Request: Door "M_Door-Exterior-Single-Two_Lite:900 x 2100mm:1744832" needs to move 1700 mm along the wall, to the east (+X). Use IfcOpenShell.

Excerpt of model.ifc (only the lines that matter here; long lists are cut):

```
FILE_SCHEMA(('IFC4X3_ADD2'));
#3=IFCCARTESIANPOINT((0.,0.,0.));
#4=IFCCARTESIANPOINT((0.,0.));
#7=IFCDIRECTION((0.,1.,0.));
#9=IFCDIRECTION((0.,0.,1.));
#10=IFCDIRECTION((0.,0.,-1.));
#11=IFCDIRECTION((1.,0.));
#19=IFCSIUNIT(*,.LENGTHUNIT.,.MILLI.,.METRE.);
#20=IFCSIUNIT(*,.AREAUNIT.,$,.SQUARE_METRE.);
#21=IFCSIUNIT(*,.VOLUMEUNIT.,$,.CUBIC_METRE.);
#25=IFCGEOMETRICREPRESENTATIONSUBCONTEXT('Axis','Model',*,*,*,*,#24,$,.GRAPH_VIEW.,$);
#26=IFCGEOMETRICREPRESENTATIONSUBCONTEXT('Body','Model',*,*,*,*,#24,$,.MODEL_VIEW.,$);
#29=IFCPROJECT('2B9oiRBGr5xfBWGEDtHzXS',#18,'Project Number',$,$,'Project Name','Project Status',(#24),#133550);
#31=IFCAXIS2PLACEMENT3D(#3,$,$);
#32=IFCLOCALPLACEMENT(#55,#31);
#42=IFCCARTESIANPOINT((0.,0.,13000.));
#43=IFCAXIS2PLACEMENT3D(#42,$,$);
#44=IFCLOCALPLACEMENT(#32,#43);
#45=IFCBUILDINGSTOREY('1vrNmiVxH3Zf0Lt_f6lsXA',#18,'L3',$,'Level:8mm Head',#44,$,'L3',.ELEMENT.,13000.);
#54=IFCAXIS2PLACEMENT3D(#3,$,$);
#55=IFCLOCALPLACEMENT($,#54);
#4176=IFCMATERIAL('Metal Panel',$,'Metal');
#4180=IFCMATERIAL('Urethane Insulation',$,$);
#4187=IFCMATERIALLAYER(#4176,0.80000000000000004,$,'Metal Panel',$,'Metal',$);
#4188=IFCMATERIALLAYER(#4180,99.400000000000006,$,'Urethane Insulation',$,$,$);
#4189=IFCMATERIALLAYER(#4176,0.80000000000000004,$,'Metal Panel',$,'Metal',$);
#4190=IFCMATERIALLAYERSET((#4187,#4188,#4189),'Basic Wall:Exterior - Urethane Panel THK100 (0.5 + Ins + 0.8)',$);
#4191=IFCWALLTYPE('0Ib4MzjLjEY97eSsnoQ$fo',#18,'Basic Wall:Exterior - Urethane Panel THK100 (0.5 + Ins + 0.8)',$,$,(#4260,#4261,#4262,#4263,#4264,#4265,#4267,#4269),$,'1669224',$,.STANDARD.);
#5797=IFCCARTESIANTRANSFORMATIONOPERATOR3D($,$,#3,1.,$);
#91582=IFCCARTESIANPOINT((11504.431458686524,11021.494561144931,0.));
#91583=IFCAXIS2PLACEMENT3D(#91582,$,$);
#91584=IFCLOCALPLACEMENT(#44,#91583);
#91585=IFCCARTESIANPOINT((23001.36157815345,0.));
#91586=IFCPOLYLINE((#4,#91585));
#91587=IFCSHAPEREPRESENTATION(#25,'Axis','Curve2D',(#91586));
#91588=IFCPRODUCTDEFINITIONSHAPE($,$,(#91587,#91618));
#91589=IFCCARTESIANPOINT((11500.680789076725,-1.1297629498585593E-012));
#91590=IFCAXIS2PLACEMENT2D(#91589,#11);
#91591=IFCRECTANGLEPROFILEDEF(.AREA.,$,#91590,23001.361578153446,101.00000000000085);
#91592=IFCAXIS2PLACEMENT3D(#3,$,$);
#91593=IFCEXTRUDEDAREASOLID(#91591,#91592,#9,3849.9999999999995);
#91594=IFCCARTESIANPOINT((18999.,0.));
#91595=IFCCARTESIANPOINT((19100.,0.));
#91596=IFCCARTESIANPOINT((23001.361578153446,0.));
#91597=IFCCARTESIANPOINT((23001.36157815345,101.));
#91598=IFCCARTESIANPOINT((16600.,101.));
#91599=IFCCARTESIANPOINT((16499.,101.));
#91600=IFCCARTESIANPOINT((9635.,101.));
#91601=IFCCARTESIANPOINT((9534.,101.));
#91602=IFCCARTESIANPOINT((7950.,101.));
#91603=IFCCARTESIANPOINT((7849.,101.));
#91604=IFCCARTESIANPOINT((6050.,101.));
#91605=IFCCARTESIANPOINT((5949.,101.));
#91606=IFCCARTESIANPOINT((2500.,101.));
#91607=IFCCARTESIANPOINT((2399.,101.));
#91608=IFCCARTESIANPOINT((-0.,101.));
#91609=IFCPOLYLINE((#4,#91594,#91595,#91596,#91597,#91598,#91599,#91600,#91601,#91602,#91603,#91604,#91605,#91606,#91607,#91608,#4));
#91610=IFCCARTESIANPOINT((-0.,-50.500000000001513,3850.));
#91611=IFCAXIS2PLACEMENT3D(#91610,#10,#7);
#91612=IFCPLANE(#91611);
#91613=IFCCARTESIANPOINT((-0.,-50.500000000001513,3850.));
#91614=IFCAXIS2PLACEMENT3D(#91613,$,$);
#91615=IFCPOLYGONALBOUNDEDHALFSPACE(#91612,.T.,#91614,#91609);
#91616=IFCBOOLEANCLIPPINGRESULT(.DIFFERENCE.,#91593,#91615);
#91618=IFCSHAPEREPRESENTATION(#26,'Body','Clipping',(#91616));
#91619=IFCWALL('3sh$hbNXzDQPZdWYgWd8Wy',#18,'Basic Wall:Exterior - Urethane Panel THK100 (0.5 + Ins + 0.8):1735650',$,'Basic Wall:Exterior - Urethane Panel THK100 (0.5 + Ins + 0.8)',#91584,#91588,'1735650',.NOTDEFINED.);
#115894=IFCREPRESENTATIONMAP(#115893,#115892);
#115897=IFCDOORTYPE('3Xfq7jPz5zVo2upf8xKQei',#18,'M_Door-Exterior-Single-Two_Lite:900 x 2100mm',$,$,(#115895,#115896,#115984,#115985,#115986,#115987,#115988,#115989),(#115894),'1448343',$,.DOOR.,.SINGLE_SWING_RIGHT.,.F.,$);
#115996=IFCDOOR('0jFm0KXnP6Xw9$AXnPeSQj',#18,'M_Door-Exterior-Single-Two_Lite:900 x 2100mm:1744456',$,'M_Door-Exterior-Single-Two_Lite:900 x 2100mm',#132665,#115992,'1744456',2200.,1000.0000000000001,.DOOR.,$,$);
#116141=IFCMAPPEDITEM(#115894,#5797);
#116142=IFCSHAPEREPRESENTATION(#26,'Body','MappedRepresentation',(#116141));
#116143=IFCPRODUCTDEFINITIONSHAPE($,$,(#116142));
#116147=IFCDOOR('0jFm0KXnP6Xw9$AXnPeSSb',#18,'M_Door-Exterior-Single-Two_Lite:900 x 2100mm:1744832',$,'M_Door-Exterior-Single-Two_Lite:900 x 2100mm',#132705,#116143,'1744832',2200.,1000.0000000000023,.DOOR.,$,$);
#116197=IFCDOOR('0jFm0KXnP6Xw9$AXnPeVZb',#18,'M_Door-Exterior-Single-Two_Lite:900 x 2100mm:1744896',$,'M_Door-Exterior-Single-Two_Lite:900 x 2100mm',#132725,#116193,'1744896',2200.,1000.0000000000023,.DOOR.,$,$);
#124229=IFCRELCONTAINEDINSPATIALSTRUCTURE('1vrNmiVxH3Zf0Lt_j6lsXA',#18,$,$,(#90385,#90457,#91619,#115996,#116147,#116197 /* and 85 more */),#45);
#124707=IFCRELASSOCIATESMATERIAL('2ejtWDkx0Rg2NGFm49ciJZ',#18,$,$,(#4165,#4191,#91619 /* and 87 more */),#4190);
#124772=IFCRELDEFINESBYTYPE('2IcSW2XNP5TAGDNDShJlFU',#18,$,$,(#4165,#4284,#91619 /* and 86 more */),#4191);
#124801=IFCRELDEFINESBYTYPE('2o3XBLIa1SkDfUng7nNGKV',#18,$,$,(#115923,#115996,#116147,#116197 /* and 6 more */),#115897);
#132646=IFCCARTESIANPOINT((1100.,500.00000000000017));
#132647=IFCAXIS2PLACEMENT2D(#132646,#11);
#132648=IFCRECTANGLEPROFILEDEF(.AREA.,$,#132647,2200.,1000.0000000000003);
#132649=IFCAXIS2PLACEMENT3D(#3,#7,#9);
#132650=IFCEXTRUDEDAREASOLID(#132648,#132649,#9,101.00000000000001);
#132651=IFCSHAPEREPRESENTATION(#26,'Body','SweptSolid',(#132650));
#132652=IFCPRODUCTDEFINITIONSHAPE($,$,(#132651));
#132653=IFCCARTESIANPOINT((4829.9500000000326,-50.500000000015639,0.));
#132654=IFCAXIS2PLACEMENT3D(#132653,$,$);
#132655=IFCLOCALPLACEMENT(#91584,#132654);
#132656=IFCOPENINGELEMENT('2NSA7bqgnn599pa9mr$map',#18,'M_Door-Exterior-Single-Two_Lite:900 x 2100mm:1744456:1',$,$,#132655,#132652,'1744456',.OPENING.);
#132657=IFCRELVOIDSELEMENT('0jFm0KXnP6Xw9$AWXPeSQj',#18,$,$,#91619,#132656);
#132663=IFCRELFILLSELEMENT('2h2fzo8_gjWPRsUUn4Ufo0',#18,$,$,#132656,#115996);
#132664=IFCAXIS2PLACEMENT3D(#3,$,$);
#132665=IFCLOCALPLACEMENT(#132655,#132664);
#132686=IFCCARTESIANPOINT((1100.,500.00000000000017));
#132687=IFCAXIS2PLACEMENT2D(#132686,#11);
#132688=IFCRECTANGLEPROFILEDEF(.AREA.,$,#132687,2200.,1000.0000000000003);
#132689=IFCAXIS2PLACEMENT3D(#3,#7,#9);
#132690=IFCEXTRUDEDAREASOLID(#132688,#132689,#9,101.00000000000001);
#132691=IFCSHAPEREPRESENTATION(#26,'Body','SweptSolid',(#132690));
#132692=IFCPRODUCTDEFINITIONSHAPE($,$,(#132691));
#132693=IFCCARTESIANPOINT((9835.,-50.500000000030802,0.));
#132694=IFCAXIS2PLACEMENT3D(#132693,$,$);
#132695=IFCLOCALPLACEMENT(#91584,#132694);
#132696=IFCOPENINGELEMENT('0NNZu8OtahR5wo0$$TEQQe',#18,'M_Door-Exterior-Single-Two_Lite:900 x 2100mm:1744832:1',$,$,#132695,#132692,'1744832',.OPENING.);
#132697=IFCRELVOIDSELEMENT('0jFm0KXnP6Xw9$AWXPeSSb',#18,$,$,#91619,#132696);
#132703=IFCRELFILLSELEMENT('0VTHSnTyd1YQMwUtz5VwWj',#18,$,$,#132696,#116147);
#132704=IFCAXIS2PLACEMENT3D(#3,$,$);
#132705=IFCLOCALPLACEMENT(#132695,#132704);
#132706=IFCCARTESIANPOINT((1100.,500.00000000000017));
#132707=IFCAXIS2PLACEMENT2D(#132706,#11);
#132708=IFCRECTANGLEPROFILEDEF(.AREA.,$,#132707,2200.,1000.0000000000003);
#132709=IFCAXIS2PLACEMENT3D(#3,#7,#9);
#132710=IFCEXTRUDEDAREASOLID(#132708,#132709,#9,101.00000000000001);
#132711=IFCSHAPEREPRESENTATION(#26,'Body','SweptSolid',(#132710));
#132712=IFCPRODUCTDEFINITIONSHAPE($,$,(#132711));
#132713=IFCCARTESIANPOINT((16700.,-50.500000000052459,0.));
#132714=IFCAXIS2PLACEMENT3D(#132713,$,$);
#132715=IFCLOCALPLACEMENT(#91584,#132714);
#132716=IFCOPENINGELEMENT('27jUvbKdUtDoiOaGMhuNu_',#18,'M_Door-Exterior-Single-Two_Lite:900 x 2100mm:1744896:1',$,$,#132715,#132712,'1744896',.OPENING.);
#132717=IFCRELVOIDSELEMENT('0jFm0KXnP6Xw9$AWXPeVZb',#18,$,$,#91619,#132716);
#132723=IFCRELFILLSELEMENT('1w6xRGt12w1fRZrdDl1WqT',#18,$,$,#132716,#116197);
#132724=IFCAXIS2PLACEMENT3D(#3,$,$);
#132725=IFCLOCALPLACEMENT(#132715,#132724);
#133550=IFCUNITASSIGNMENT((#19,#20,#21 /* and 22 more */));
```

```python
import ifcopenshell
import ifcopenshell.api.geometry
import ifcopenshell.util.placement
import ifcopenshell.util.unit

model = ifcopenshell.open("model.ifc")
unit_scale = ifcopenshell.util.unit.calculate_unit_scale(model)

door = model.by_guid("0jFm0KXnP6Xw9$AXnPeSSb")
opening = door.FillsVoids[0].RelatingOpeningElement
wall = opening.VoidsElements[0].RelatingBuildingElement

wall_matrix = ifcopenshell.util.placement.get_local_placement(wall.ObjectPlacement)
shift = wall_matrix[:3, 0] * 1.7 / unit_scale
before = ifcopenshell.util.placement.get_local_placement(door.ObjectPlacement)[:3, 3].copy()

# The door is placed relative to its opening, so it follows when the opening moves.
matrix = ifcopenshell.util.placement.get_local_placement(opening.ObjectPlacement)
matrix[:3, 3] += shift
ifcopenshell.api.geometry.edit_object_placement(
    model, product=opening, matrix=matrix, is_si=False, should_transform_children=True
)

after = ifcopenshell.util.placement.get_local_placement(door.ObjectPlacement)[:3, 3]
print("door moved by", (after - before).round(3) + 0.0)

model.write("model_edited.ifc")
```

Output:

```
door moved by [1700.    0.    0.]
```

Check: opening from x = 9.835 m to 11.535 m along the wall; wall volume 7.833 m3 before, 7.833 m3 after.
